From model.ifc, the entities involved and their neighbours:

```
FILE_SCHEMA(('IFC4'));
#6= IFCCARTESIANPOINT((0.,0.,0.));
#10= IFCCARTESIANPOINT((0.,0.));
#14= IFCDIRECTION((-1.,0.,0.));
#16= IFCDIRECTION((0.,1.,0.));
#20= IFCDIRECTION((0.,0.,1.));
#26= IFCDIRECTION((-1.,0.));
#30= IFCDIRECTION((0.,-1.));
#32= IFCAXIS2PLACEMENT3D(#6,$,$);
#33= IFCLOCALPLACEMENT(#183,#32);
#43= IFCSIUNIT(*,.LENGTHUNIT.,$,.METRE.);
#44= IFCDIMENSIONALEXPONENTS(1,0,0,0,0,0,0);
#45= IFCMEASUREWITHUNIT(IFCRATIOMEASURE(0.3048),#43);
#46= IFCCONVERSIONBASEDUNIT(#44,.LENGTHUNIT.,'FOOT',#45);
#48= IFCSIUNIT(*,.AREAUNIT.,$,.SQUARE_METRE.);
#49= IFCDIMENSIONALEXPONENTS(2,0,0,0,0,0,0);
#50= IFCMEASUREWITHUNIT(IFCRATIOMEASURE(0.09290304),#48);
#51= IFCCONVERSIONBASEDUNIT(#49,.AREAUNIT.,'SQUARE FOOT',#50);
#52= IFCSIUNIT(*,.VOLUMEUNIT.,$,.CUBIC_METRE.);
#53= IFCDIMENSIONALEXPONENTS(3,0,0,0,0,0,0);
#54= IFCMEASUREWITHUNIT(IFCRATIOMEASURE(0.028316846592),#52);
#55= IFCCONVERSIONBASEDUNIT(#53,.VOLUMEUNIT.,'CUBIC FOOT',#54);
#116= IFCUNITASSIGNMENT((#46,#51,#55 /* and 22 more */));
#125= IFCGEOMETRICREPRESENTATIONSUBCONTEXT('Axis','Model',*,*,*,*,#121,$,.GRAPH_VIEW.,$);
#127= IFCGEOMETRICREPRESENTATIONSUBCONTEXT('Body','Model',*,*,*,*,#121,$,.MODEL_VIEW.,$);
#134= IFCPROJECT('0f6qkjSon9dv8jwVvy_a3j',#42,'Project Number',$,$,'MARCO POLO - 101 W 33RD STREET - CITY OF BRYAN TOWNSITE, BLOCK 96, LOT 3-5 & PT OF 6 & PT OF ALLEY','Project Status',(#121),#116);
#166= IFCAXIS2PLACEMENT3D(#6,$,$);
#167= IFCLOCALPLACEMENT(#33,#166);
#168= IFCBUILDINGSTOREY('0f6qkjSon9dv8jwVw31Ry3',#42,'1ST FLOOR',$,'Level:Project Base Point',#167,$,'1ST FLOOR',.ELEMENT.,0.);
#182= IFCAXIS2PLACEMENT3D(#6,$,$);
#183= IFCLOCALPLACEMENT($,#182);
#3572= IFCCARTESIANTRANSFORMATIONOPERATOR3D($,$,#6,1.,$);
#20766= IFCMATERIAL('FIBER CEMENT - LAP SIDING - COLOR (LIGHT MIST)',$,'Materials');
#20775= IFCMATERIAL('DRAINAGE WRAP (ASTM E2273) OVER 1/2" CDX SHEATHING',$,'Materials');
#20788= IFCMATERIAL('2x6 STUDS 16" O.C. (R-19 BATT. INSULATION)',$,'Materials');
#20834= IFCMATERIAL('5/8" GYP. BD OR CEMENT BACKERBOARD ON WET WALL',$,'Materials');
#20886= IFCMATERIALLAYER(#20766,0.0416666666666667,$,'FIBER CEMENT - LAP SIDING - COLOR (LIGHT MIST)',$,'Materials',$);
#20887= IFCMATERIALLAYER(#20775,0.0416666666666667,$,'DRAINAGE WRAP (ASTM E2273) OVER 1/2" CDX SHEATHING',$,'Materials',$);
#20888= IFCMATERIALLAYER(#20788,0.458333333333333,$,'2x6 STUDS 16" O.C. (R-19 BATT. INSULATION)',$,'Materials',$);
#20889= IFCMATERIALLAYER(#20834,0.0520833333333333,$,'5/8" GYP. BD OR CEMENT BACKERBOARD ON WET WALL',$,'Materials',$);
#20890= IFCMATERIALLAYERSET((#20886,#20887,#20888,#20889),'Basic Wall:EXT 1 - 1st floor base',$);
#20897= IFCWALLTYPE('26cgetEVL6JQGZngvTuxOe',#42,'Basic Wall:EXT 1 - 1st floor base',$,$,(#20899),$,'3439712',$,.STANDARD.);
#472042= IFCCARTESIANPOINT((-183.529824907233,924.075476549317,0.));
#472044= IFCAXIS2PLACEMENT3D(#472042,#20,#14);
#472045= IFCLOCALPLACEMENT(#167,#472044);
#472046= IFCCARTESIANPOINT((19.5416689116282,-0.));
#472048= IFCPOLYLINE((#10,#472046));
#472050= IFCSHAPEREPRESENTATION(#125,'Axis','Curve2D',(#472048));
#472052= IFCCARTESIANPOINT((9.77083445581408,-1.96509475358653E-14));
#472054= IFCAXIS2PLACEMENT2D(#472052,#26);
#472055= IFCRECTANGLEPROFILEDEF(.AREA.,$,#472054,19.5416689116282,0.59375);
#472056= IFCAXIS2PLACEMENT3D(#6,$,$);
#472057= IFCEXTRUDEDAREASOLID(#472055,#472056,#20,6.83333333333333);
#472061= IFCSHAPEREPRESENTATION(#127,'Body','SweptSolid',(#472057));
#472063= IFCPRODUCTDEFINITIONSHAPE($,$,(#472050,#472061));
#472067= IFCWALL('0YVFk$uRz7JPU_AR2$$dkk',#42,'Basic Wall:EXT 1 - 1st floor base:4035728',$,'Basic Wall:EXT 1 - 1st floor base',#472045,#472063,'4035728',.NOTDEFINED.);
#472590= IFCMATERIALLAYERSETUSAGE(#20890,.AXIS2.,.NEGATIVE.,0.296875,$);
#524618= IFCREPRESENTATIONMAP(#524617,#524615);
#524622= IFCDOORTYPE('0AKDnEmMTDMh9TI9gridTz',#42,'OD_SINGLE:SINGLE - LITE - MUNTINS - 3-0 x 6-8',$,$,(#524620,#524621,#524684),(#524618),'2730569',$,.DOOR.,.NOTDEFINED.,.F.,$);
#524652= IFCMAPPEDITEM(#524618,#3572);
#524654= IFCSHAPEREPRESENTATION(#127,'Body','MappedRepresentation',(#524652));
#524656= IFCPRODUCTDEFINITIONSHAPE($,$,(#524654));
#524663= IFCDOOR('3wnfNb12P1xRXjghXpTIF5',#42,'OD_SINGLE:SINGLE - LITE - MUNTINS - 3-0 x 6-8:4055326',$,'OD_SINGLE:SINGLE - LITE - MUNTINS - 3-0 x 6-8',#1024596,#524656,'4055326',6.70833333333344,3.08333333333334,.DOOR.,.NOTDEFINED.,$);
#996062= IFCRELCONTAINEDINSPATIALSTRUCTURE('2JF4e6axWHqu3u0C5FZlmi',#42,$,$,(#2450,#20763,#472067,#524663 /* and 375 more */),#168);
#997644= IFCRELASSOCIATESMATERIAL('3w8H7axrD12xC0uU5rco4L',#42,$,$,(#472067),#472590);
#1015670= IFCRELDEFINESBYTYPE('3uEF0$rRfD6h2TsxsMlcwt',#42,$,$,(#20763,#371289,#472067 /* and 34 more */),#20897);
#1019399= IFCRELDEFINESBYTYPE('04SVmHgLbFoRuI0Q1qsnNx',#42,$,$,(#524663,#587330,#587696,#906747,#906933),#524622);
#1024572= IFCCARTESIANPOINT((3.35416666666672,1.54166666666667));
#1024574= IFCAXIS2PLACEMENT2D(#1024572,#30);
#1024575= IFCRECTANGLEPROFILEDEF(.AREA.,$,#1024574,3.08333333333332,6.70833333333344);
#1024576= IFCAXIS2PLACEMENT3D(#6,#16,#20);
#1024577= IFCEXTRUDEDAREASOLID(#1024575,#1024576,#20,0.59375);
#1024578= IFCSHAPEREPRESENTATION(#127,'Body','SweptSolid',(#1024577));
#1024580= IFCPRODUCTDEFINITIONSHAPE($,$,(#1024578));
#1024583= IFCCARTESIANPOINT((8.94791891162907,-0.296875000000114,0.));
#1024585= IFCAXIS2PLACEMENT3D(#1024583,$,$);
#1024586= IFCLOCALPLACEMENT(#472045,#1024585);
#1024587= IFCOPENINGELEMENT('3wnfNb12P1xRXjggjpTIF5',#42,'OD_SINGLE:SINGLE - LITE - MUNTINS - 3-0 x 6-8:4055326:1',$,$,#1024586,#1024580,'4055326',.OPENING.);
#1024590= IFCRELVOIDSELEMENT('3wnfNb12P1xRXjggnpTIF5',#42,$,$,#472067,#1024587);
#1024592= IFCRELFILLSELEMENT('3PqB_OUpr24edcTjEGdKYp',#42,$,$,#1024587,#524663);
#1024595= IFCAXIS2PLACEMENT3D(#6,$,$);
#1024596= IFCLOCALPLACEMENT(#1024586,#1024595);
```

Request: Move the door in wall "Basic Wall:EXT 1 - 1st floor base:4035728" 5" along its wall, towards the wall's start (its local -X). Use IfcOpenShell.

```python
import ifcopenshell
import ifcopenshell.api.geometry
import ifcopenshell.util.placement
import ifcopenshell.util.unit

model = ifcopenshell.open("model.ifc")
unit_scale = ifcopenshell.util.unit.calculate_unit_scale(model)

door = model.by_id(524663)
opening = door.FillsVoids[0].RelatingOpeningElement
wall = opening.VoidsElements[0].RelatingBuildingElement

wall_matrix = ifcopenshell.util.placement.get_local_placement(wall.ObjectPlacement)
shift = wall_matrix[:3, 0] * -5 * 0.0254 / unit_scale
before = ifcopenshell.util.placement.get_local_placement(door.ObjectPlacement)[:3, 3].copy()

# The door is placed relative to its opening, so it follows when the opening moves.
matrix = ifcopenshell.util.placement.get_local_placement(opening.ObjectPlacement)
matrix[:3, 3] += shift
ifcopenshell.api.geometry.edit_object_placement(
    model, product=opening, matrix=matrix, is_si=False, should_transform_children=True
)

after = ifcopenshell.util.placement.get_local_placement(door.ObjectPlacement)[:3, 3]
print("door moved by", (after - before).round(3) + 0.0)

model.write("model-out.ifc")
```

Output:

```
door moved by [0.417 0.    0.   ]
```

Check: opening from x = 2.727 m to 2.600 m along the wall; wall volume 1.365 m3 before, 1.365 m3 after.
